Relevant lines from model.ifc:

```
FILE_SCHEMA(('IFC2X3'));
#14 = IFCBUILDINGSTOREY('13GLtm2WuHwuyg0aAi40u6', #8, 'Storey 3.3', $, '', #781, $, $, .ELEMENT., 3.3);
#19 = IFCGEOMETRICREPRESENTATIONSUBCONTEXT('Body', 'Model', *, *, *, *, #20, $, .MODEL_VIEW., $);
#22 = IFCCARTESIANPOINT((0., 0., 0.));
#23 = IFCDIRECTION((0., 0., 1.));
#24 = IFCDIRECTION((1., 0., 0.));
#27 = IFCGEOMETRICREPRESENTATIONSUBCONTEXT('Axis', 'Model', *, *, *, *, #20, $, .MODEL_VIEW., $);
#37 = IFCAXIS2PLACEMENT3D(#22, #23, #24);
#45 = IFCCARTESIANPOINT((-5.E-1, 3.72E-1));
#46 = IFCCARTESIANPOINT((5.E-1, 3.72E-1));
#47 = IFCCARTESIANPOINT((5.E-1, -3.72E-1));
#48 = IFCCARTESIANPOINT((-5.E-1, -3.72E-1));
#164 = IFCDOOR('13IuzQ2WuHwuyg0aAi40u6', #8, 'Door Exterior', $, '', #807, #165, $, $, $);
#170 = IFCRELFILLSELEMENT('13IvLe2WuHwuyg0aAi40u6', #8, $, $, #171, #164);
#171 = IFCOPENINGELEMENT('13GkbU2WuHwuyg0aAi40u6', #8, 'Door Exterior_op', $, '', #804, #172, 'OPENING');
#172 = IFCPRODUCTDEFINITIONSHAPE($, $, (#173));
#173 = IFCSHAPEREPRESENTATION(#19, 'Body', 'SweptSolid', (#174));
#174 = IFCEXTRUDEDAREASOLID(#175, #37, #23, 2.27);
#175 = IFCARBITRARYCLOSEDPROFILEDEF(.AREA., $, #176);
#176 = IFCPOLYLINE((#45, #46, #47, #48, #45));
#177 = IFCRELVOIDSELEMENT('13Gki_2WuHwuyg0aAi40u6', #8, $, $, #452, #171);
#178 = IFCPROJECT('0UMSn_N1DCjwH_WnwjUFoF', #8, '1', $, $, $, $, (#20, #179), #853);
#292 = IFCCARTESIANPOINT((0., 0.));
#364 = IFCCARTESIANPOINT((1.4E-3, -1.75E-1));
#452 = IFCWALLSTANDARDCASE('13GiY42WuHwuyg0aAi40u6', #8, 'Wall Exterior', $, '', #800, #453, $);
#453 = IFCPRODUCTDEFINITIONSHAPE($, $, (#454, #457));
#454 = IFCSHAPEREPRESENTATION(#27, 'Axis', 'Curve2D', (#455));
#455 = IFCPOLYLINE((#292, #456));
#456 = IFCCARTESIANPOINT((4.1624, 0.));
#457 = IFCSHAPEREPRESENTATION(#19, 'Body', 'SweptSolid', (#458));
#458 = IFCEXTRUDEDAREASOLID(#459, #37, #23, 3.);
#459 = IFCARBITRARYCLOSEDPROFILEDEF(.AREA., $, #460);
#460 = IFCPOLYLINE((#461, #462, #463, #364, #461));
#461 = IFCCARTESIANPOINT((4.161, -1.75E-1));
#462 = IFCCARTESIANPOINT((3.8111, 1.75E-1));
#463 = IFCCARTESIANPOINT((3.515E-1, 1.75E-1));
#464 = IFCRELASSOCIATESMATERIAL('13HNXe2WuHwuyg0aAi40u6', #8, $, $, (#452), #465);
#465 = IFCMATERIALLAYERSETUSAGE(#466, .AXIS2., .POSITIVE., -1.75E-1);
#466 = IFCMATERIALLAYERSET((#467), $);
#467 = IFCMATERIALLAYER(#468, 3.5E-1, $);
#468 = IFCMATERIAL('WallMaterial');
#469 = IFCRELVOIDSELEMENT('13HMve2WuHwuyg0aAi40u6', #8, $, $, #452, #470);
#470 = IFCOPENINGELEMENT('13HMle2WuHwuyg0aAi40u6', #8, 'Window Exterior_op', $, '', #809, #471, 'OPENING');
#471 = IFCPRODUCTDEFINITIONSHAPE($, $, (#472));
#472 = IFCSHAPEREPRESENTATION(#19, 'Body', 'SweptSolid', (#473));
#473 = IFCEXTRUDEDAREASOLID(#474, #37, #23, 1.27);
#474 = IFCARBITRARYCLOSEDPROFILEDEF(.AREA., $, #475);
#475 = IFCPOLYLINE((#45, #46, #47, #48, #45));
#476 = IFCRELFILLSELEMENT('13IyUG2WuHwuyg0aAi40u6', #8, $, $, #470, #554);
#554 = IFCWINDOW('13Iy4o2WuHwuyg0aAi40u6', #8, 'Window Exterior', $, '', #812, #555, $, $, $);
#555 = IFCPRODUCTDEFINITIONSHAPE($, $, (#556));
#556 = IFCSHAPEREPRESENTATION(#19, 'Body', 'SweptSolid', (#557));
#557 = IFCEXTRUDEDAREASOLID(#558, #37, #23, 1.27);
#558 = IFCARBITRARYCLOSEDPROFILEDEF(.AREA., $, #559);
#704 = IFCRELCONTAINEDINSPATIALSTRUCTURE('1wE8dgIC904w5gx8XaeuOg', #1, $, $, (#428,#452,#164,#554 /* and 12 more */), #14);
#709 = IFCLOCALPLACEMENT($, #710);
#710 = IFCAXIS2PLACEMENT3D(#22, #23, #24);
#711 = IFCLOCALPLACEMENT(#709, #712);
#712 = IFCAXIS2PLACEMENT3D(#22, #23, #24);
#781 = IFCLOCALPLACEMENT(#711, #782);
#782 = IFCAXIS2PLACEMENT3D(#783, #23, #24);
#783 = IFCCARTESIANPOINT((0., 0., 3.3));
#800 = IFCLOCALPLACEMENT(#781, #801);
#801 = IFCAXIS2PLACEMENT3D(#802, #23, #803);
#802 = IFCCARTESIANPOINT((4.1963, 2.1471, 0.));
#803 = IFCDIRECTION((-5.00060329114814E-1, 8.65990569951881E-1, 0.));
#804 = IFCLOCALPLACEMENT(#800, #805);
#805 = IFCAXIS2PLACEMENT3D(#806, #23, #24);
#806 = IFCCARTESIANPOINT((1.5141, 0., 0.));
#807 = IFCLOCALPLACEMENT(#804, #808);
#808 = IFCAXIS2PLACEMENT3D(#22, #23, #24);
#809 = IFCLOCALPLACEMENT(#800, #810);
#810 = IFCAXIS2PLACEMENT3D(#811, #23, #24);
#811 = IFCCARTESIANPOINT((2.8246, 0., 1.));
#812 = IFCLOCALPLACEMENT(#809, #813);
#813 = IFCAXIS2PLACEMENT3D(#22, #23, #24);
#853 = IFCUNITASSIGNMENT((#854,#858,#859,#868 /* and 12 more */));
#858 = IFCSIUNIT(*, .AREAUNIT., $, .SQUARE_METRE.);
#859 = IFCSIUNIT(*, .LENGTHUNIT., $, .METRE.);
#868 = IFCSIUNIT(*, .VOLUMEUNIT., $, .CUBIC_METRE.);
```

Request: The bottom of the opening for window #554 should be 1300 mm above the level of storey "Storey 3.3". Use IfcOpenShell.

```python
import numpy as np
import ifcopenshell
import ifcopenshell.api.geometry
import ifcopenshell.geom
import ifcopenshell.util.element
import ifcopenshell.util.placement
import ifcopenshell.util.shape
import ifcopenshell.util.unit

model = ifcopenshell.open("model.ifc")
unit_scale = ifcopenshell.util.unit.calculate_unit_scale(model)

window = model.by_guid("13Iy4o2WuHwuyg0aAi40u6")
opening = window.FillsVoids[0].RelatingOpeningElement
storey = ifcopenshell.util.element.get_container(window, ifc_class="IfcBuildingStorey")
level = ifcopenshell.util.placement.get_local_placement(storey.ObjectPlacement)[2, 3]

# The opening's origin need not be at the sill, so measure its lowest point.
shape = ifcopenshell.geom.create_shape(ifcopenshell.geom.settings(), opening)
bottom = ifcopenshell.util.shape.get_shape_bottom_elevation(shape, shape.geometry) / unit_scale
dz = level + 1.3 - bottom

shift = np.array([0.0, 0.0, dz])
# The window is placed relative to its opening, so it follows when the opening moves.
matrix = ifcopenshell.util.placement.get_local_placement(opening.ObjectPlacement)
matrix[:3, 3] += shift
ifcopenshell.api.geometry.edit_object_placement(
    model, product=opening, matrix=matrix, is_si=False, should_transform_children=True
)

print(f"moved by {dz * unit_scale:+.3f} m")

model.write("model-out.ifc")
```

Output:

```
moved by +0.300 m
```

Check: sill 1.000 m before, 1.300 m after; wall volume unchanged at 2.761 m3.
